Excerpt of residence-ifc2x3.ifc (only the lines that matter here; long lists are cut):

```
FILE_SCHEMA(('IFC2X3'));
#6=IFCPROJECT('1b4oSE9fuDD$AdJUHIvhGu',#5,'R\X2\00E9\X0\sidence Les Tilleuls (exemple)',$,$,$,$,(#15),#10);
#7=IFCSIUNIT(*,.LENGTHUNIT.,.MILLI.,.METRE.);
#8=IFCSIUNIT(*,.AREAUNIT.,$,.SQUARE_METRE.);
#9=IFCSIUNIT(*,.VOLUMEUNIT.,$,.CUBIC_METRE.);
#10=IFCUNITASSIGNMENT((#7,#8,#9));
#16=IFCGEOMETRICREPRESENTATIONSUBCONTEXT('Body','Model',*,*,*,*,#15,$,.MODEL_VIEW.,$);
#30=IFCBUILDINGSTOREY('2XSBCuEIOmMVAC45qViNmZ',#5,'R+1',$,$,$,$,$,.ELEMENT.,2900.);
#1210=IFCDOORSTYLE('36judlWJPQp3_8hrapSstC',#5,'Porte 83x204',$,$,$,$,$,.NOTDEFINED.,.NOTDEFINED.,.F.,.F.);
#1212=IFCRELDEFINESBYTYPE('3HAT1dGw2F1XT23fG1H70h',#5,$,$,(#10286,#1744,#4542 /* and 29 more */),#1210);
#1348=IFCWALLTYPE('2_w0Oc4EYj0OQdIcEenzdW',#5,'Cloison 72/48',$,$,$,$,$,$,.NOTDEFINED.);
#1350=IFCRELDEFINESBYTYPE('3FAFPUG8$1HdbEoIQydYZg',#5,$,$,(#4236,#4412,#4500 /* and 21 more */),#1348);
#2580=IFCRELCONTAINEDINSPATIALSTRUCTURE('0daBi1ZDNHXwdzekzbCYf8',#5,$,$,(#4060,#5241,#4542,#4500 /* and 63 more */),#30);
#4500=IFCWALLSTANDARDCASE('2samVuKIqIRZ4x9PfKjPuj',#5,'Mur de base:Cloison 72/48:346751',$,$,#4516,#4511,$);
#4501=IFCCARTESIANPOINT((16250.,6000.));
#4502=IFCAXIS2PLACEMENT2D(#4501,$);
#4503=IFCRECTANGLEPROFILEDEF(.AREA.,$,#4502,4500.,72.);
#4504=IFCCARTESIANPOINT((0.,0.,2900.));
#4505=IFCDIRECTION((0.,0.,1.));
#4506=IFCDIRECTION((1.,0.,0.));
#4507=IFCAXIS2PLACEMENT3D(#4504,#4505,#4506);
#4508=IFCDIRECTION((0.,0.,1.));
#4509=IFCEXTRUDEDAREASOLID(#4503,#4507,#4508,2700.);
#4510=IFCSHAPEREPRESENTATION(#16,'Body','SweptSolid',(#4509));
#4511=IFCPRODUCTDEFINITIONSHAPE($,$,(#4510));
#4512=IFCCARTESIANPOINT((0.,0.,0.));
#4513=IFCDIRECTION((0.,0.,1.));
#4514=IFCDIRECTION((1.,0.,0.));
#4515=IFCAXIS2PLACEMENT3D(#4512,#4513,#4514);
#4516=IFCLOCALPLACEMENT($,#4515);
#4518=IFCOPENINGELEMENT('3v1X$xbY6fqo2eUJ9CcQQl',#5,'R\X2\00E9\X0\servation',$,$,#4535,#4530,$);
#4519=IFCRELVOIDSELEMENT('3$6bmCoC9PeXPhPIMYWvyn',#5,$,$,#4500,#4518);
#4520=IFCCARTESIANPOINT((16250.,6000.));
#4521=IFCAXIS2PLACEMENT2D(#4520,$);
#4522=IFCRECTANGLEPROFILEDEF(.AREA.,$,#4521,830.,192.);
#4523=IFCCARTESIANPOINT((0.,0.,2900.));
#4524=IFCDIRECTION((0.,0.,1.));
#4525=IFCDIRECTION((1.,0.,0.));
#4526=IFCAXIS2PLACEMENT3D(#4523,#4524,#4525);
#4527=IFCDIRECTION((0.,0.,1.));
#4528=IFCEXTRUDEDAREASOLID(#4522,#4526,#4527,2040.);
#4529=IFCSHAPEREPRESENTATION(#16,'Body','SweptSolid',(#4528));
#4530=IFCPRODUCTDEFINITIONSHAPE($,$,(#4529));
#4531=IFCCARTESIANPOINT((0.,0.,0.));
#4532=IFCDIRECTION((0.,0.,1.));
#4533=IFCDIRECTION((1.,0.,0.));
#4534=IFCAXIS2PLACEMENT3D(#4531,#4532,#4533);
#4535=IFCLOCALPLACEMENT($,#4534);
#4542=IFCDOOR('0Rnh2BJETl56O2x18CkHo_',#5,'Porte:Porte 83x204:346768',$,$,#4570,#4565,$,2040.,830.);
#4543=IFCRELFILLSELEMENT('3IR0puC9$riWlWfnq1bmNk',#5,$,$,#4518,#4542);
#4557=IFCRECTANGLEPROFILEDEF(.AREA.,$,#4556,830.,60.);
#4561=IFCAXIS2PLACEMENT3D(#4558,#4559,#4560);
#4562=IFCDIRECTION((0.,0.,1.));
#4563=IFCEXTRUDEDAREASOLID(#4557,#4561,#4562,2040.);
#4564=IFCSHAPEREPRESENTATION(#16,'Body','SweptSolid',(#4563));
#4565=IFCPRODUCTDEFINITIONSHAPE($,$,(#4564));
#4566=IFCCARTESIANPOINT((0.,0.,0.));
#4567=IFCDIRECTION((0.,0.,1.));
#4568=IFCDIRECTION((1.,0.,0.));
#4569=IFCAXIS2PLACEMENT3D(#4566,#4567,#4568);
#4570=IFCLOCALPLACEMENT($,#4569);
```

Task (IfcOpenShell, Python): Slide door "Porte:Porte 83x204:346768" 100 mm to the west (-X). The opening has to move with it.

```python
import ifcopenshell
import ifcopenshell.api.geometry
import ifcopenshell.util.placement

model = ifcopenshell.open("residence-ifc2x3.ifc")

door = model.by_id(4542)
opening = door.FillsVoids[0].RelatingOpeningElement
wall = opening.VoidsElements[0].RelatingBuildingElement

wall_matrix = ifcopenshell.util.placement.get_local_placement(wall.ObjectPlacement)
shift = wall_matrix[:3, 0] * -100.0
before = ifcopenshell.util.placement.get_local_placement(door.ObjectPlacement)[:3, 3].copy()

# The door is not placed relative to its opening, so move both.
for product in (opening, door):
    matrix = ifcopenshell.util.placement.get_local_placement(product.ObjectPlacement)
    matrix[:3, 3] += shift
    ifcopenshell.api.geometry.edit_object_placement(model, product=product, matrix=matrix, is_si=False)

after = ifcopenshell.util.placement.get_local_placement(door.ObjectPlacement)[:3, 3]
print("door moved by", (after - before).round(3) + 0.0)

model.write("residence-ifc2x3_edited.ifc")
```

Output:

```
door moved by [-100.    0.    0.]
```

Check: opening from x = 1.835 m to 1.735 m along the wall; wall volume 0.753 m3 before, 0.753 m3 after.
